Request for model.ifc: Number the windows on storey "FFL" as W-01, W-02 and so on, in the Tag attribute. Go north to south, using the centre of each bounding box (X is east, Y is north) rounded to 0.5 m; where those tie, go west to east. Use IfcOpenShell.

First a look at what the model holds.

```python
import ifcopenshell
import ifcopenshell.util.element
import ifcopenshell.util.placement

model = ifcopenshell.open("model.ifc")
print(model.schema)
storey = next(s for s in model.by_type("IfcBuildingStorey") if s.Name == "FFL")
windows = [e for e in ifcopenshell.util.element.get_decomposition(storey) if e.is_a("IfcWindow")]
for e in sorted(windows, key=lambda e: e.id()):
    origin = ifcopenshell.util.placement.get_local_placement(e.ObjectPlacement)[:3, 3]
    print(e.id(), e.Tag, e.Name, origin.round(2) + 0.0, sep=" | ")
```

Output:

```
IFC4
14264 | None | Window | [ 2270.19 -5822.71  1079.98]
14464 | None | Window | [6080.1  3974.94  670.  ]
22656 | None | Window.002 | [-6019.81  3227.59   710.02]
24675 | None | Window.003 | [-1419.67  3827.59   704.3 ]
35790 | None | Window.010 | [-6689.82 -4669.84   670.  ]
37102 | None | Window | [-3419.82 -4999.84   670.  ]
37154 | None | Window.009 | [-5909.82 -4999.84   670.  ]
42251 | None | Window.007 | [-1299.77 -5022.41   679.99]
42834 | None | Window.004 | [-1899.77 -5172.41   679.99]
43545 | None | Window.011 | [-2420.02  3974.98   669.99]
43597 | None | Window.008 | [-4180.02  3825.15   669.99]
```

```python
import ifcopenshell
import ifcopenshell.geom
import ifcopenshell.util.element
import ifcopenshell.util.shape

model = ifcopenshell.open("model.ifc")
settings = ifcopenshell.geom.settings()
settings.set("use-world-coords", True)


def centre(element):
    shape = ifcopenshell.geom.create_shape(settings, element)
    return ifcopenshell.util.shape.get_bbox_centroid(shape.geometry)


storey = next(s for s in model.by_type("IfcBuildingStorey") if s.Name == "FFL")
windows = [e for e in ifcopenshell.util.element.get_decomposition(storey) if e.is_a("IfcWindow")]

# Insertion points can sit at a corner or the storey origin, so sort by the geometry (in metres).
centres = {e: centre(e) for e in windows}
windows.sort(key=lambda e: (-round(centres[e][1] / 0.5), centres[e][0]))

for i, e in enumerate(windows, start=1):
    number = f"W-{i:02d}"
    e.Tag = number
    print(e.id(), number)

model.write("model_v2.ifc")
```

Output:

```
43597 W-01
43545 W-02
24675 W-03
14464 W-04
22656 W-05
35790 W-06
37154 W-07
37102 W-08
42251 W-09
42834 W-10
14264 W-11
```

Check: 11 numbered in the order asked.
